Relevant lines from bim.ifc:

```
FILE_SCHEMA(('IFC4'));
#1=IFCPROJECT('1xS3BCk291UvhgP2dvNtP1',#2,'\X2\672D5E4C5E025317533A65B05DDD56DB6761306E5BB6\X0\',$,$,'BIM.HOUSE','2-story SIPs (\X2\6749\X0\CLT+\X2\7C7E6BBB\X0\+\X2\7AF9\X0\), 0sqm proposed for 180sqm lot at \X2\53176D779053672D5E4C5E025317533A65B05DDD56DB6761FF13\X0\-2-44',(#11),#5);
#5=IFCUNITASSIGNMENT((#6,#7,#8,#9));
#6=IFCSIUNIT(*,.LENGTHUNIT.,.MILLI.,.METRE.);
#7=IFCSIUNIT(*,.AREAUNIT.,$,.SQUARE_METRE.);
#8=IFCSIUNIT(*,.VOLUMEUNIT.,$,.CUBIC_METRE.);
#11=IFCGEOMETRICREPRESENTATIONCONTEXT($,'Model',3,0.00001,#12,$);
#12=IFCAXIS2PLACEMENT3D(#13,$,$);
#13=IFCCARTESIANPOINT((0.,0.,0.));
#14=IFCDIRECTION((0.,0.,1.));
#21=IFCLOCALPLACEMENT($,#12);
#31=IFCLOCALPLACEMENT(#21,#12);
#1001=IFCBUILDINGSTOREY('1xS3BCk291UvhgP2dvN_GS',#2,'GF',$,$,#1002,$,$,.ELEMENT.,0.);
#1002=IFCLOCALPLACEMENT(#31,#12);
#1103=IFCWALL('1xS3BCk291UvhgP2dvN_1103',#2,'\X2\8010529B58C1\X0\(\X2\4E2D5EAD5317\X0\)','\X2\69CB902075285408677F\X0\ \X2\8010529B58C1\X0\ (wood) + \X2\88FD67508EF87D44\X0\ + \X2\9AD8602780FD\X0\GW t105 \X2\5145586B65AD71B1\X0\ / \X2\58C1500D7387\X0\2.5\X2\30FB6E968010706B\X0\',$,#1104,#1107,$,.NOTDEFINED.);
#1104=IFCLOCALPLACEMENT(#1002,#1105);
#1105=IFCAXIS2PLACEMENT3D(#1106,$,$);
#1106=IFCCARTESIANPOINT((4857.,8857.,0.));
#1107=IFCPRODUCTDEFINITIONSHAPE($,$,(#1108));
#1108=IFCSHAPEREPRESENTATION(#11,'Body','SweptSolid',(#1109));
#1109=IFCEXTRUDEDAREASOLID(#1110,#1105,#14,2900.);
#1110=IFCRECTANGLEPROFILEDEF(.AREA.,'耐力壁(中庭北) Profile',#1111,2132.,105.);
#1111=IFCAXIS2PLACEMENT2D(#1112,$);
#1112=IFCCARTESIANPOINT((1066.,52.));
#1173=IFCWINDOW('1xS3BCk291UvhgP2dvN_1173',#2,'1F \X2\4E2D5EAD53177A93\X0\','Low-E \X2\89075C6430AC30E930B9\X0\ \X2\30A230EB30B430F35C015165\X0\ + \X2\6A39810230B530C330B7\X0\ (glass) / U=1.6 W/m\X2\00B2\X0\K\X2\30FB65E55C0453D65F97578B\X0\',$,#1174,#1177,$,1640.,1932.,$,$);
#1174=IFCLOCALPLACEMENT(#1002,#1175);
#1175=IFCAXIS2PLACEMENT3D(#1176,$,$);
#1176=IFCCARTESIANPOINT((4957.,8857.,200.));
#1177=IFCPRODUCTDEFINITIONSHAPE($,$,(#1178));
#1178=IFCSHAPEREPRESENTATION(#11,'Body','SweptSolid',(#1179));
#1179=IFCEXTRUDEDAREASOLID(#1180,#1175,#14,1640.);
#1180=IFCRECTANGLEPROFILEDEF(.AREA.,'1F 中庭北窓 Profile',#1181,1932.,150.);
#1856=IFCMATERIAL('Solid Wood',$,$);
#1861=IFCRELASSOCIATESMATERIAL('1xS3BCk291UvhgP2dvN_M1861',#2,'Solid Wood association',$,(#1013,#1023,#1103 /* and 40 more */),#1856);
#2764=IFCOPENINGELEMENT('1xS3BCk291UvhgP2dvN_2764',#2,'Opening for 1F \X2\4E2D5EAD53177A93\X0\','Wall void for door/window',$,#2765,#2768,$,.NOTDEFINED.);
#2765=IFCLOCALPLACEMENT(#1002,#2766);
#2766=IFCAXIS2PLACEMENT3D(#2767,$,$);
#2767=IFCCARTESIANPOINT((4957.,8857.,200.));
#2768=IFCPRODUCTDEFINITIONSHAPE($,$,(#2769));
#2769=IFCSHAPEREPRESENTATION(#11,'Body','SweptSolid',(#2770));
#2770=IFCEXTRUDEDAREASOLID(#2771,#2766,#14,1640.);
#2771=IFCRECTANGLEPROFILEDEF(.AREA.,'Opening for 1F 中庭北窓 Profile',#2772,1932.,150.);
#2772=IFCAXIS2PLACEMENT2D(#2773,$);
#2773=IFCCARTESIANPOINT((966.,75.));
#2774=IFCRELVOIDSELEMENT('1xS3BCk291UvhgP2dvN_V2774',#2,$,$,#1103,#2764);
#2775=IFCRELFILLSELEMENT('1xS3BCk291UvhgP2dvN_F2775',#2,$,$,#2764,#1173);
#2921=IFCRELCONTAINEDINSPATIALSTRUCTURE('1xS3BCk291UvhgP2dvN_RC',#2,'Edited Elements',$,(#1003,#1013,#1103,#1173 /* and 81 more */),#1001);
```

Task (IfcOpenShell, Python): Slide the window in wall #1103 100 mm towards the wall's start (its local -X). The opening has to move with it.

```python
import ifcopenshell
import ifcopenshell.api.geometry
import ifcopenshell.util.placement

model = ifcopenshell.open("bim.ifc")

window = model.by_guid("1xS3BCk291UvhgP2dvN_1173")
opening = window.FillsVoids[0].RelatingOpeningElement
wall = opening.VoidsElements[0].RelatingBuildingElement

wall_matrix = ifcopenshell.util.placement.get_local_placement(wall.ObjectPlacement)
shift = wall_matrix[:3, 0] * -100.0
before = ifcopenshell.util.placement.get_local_placement(window.ObjectPlacement)[:3, 3].copy()

# The window is not placed relative to its opening, so move both.
for product in (opening, window):
    matrix = ifcopenshell.util.placement.get_local_placement(product.ObjectPlacement)
    matrix[:3, 3] += shift
    ifcopenshell.api.geometry.edit_object_placement(model, product=product, matrix=matrix, is_si=False)

after = ifcopenshell.util.placement.get_local_placement(window.ObjectPlacement)[:3, 3]
print("window moved by", (after - before).round(3) + 0.0)

model.write("bim-out.ifc")
```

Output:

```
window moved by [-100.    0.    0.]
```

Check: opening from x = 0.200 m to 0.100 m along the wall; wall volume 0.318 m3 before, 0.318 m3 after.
